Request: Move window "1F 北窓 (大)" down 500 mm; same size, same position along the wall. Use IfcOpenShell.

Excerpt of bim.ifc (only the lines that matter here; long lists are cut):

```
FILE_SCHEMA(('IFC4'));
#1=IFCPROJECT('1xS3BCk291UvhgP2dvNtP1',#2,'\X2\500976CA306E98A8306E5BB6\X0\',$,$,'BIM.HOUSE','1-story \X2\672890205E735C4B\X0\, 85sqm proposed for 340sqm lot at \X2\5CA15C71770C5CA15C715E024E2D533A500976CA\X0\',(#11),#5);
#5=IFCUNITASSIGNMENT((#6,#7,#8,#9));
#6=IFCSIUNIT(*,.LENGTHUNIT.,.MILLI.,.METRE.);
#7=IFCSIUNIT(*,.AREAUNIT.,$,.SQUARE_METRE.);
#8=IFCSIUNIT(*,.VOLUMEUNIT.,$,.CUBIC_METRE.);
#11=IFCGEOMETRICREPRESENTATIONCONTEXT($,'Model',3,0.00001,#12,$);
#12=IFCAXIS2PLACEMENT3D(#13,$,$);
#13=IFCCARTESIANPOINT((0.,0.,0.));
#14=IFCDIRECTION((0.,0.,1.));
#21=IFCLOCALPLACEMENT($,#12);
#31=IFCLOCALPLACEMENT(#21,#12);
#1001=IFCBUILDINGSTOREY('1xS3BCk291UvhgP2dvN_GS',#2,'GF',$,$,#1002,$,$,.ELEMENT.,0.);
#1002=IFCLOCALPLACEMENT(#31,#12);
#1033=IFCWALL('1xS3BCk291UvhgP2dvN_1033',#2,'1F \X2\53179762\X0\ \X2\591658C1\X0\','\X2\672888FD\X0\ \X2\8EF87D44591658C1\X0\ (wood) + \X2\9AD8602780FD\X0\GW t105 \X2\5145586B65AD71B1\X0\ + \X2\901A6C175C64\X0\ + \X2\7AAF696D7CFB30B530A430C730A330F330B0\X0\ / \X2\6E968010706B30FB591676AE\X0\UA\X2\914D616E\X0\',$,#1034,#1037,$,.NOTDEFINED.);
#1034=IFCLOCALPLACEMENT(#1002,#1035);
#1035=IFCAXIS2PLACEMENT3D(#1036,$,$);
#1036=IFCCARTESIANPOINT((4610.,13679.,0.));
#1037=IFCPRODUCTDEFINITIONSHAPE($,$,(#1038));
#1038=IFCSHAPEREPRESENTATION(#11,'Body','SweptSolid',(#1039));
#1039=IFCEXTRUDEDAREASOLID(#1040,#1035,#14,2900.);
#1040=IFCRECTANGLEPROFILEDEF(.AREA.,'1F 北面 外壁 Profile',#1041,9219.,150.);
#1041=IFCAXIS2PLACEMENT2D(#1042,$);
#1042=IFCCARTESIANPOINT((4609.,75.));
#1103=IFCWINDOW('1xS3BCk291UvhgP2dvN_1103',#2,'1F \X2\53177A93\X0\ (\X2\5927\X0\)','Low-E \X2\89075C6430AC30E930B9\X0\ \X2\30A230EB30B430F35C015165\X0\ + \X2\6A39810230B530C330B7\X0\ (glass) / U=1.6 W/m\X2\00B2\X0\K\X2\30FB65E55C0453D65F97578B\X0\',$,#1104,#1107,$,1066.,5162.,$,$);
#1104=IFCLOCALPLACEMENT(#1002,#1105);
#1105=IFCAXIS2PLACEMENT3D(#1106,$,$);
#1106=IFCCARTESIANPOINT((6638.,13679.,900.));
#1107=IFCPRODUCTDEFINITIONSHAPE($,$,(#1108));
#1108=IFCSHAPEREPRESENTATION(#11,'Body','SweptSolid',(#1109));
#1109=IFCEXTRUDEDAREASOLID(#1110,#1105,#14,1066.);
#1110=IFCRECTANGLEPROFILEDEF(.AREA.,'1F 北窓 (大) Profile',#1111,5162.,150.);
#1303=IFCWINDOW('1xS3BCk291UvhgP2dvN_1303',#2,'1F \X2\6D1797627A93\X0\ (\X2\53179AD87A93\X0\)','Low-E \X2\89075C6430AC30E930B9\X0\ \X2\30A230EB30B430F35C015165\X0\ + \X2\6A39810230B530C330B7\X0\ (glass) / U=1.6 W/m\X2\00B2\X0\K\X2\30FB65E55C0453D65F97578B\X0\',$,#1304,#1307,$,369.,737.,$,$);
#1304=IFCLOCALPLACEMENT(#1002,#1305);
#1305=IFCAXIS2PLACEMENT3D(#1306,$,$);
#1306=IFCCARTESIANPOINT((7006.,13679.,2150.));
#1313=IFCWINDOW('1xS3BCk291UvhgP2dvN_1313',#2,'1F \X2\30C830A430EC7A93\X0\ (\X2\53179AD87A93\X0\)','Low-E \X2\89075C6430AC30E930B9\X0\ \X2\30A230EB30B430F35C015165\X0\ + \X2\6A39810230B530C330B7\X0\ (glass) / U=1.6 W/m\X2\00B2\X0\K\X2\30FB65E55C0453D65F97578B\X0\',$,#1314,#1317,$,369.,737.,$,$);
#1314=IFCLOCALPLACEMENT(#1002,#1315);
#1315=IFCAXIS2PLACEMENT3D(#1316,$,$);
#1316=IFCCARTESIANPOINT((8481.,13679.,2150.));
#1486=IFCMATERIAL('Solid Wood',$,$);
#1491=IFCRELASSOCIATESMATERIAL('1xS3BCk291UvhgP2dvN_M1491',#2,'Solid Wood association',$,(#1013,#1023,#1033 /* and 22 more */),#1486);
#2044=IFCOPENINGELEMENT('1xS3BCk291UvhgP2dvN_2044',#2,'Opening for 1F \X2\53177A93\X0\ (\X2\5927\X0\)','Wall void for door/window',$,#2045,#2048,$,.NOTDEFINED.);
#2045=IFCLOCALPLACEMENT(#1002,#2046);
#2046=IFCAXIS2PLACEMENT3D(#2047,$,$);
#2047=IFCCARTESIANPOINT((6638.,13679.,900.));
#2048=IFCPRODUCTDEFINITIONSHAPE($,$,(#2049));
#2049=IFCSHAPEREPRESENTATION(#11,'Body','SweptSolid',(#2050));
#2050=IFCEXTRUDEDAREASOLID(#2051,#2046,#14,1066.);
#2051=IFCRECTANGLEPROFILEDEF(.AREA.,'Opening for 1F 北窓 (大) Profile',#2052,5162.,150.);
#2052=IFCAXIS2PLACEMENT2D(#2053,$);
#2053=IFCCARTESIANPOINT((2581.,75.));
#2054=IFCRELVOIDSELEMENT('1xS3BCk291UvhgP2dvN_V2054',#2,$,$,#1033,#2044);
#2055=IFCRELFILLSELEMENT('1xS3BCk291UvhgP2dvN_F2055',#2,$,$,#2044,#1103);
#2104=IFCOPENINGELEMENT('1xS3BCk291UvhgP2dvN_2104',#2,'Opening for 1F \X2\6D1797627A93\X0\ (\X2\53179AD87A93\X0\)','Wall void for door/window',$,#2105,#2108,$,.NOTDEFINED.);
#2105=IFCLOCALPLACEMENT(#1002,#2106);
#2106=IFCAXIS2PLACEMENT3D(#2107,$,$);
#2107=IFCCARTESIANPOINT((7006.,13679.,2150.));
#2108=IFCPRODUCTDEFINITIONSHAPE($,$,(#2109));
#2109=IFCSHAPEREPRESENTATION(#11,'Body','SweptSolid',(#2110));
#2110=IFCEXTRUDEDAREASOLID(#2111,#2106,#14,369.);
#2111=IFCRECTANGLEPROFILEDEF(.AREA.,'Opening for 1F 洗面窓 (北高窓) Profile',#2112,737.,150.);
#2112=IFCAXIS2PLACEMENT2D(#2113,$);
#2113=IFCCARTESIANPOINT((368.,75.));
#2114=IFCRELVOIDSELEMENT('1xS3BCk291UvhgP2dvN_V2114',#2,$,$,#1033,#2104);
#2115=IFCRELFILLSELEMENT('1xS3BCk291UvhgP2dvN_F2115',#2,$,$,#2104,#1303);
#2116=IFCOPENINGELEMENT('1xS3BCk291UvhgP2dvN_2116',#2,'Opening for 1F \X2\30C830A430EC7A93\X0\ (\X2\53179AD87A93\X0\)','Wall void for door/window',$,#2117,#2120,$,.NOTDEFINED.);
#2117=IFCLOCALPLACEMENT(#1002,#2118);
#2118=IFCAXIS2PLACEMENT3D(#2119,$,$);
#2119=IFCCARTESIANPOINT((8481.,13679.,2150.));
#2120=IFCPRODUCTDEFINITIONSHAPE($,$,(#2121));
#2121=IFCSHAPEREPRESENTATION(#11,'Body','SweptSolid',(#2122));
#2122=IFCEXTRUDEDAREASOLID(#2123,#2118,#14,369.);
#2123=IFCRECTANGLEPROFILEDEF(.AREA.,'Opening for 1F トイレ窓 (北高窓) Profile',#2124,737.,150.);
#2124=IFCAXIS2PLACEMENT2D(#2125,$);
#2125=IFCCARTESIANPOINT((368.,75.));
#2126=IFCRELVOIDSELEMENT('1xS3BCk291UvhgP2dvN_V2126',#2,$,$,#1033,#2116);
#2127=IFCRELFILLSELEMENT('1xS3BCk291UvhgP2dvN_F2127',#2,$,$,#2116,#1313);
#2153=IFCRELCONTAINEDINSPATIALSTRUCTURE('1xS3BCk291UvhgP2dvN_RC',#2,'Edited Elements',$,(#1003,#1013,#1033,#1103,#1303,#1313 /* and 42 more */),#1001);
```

```python
import numpy as np
import ifcopenshell
import ifcopenshell.api.geometry
import ifcopenshell.util.placement
import ifcopenshell.util.unit

model = ifcopenshell.open("bim.ifc")
unit_scale = ifcopenshell.util.unit.calculate_unit_scale(model)

window = model.by_guid("1xS3BCk291UvhgP2dvN_1103")
opening = window.FillsVoids[0].RelatingOpeningElement
dz = -500.0

shift = np.array([0.0, 0.0, dz])
# The window is not placed relative to its opening, so move both.
for product in (opening, window):
    matrix = ifcopenshell.util.placement.get_local_placement(product.ObjectPlacement)
    matrix[:3, 3] += shift
    ifcopenshell.api.geometry.edit_object_placement(model, product=product, matrix=matrix, is_si=False)

print(f"moved by {dz * unit_scale:+.3f} m")

model.write("bim_rev.ifc")
```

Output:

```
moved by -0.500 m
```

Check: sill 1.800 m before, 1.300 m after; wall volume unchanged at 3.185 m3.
